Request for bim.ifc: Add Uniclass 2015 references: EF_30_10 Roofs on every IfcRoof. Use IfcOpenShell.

First a look at what the model holds.

```python
import ifcopenshell

model = ifcopenshell.open("bim.ifc")
print(model.schema)
print("classifications:", [c.Name for c in model.by_type("IfcClassification")])
for ifc_class in ("IfcDoor", "IfcRoof", "IfcStair", "IfcWall", "IfcWindow"):
    print(ifc_class, len(model.by_type(ifc_class)))
```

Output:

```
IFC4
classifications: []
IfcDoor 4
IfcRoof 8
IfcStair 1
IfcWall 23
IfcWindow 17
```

```python
import ifcopenshell
import ifcopenshell.api.classification

model = ifcopenshell.open("bim.ifc")

system = ifcopenshell.api.classification.add_classification(model, classification="Uniclass 2015")

codes = {
    "IfcRoof": ("EF_30_10", "Roofs"),
}
for ifc_class, (code, name) in codes.items():
    products = model.by_type(ifc_class)
    ifcopenshell.api.classification.add_reference(
        model, products=products, classification=system, identification=code, name=name
    )
    print(code, len(products))

model.write("bim-out.ifc")
```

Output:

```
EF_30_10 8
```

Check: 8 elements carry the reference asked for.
